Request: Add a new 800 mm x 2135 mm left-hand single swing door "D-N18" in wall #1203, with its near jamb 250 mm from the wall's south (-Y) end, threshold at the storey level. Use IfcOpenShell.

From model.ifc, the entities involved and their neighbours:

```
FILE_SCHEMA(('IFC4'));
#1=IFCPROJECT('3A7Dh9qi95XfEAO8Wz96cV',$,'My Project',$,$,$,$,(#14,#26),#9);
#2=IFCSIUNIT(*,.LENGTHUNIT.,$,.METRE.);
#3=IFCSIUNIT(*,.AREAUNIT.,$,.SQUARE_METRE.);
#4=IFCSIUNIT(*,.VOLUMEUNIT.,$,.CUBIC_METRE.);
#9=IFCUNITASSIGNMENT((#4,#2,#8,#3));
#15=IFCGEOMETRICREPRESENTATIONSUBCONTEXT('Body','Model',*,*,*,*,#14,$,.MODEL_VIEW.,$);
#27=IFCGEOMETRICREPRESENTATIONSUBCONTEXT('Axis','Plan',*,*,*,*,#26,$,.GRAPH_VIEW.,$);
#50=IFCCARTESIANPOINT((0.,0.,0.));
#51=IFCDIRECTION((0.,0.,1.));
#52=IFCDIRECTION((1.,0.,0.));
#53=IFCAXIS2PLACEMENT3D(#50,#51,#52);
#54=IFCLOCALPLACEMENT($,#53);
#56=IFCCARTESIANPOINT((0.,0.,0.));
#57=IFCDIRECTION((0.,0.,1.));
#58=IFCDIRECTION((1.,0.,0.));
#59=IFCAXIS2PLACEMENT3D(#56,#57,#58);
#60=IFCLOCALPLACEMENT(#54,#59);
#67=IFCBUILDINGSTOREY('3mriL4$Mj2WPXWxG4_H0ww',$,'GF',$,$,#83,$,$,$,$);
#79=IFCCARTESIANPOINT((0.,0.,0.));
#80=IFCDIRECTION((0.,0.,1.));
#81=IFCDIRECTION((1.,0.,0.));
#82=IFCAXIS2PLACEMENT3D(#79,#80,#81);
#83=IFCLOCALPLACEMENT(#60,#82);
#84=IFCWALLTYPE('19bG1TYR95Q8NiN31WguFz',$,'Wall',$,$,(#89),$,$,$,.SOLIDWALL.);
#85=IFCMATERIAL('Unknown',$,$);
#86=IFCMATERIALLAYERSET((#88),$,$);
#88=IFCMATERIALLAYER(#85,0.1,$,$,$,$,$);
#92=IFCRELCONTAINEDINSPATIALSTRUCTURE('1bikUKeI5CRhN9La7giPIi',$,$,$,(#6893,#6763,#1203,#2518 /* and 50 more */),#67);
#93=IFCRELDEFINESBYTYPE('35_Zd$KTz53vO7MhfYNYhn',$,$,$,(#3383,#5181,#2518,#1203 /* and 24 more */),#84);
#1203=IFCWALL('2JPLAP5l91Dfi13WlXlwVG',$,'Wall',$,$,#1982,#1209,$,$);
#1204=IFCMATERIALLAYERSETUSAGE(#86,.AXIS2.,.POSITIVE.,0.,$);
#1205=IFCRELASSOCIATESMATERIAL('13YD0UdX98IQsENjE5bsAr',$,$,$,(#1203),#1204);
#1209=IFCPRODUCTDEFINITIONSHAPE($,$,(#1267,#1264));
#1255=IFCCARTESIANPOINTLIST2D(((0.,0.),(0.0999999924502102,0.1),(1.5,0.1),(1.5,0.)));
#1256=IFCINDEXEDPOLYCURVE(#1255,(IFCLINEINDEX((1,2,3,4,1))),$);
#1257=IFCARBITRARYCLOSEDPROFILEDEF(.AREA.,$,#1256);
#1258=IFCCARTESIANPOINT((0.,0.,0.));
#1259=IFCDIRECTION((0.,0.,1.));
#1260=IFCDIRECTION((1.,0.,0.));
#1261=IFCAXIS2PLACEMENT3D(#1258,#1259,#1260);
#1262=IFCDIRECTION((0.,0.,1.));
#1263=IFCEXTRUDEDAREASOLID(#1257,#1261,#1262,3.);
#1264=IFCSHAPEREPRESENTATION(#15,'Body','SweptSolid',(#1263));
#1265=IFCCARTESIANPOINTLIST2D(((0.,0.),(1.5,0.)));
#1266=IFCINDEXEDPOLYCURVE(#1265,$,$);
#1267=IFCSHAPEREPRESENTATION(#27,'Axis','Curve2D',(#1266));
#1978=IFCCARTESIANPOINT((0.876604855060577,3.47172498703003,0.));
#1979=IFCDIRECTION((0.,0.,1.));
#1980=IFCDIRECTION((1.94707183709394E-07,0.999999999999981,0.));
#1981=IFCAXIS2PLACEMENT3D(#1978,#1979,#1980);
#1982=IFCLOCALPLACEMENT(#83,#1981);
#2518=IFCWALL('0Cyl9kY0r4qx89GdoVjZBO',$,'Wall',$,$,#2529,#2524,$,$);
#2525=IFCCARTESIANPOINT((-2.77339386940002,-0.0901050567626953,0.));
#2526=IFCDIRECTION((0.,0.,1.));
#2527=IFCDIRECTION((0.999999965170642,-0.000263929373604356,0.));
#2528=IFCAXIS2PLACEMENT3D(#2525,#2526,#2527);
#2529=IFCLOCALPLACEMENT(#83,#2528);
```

```python
import numpy as np
import ifcopenshell
import ifcopenshell.api.feature
import ifcopenshell.api.geometry
import ifcopenshell.api.root
import ifcopenshell.api.spatial
import ifcopenshell.geom
import ifcopenshell.util.element
import ifcopenshell.util.placement
import ifcopenshell.util.representation
import ifcopenshell.util.shape
import ifcopenshell.util.unit

model = ifcopenshell.open("model.ifc")
unit_scale = ifcopenshell.util.unit.calculate_unit_scale(model)
settings = ifcopenshell.geom.settings()


def volume(element):
    """Net volume in cubic metres, openings subtracted."""
    shape = ifcopenshell.geom.create_shape(settings, element)
    return ifcopenshell.util.shape.get_volume(shape.geometry)


wall = model.by_guid("2JPLAP5l91Dfi13WlXlwVG")
storey = ifcopenshell.util.element.get_container(wall, ifc_class="IfcBuildingStorey")
context = ifcopenshell.util.representation.get_context(model, "Model", "Body", "MODEL_VIEW")
before = volume(wall)

width, height, from_end, sill = 0.8, 2.135, 0.25, 0.0  # metres

# The wall runs along its own X axis, and the end named is its -X end.
wall_shape = ifcopenshell.geom.create_shape(settings, wall)
x, y, z = ifcopenshell.util.shape.get_vertices(wall_shape.geometry).T
start = x.min() + from_end
face, thickness = float(y.min()), float(y.max() - y.min())
wall_matrix = ifcopenshell.util.placement.get_local_placement(wall.ObjectPlacement)
level = ifcopenshell.util.placement.get_local_placement(storey.ObjectPlacement)[2, 3]


def in_wall(x, y):
    """Placement at x, y metres in the wall's axes, at sill height."""
    matrix = wall_matrix.copy()
    matrix[:, 3] = wall_matrix @ np.array([x / unit_scale, y / unit_scale, 0.0, 1.0])
    matrix[2, 3] = level + sill / unit_scale
    return matrix


# Opening: a box that overshoots both wall faces by 50 mm.
opening = ifcopenshell.api.root.create_entity(model, ifc_class="IfcOpeningElement", predefined_type="OPENING")
box = ifcopenshell.api.geometry.add_wall_representation(
    model, context=context, length=width, height=height, thickness=thickness + 0.1
)
ifcopenshell.api.geometry.assign_representation(model, product=opening, representation=box)
ifcopenshell.api.geometry.edit_object_placement(model, product=opening, matrix=in_wall(start, face - 0.05), is_si=False)
ifcopenshell.api.feature.add_feature(model, feature=opening, element=wall)

door = ifcopenshell.api.root.create_entity(model, ifc_class="IfcDoor", name="D-N18", predefined_type="DOOR")
door.OverallWidth, door.OverallHeight = width / unit_scale, height / unit_scale
door.OperationType = "SINGLE_SWING_LEFT"
body = ifcopenshell.api.geometry.add_door_representation(
    model,
    context=context,
    overall_width=door.OverallWidth,
    overall_height=door.OverallHeight,
    operation_type="SINGLE_SWING_LEFT",
    lining_properties={"LiningDepth": thickness / unit_scale, "ThresholdDepth": thickness / unit_scale},
)
ifcopenshell.api.geometry.assign_representation(model, product=door, representation=body)
ifcopenshell.api.spatial.assign_container(model, products=[door], relating_structure=storey)
ifcopenshell.api.feature.add_filling(model, opening=opening, element=door)

# The lining spans the wall, so the door starts at the wall face.
ifcopenshell.api.geometry.edit_object_placement(model, product=door, matrix=in_wall(start, face), is_si=False)

after = volume(wall)

print(f"wall volume {before:.3f} -> {after:.3f} m3")

model.write("model_v2.ifc")
```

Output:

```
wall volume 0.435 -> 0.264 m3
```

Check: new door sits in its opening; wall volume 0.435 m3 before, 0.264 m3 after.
